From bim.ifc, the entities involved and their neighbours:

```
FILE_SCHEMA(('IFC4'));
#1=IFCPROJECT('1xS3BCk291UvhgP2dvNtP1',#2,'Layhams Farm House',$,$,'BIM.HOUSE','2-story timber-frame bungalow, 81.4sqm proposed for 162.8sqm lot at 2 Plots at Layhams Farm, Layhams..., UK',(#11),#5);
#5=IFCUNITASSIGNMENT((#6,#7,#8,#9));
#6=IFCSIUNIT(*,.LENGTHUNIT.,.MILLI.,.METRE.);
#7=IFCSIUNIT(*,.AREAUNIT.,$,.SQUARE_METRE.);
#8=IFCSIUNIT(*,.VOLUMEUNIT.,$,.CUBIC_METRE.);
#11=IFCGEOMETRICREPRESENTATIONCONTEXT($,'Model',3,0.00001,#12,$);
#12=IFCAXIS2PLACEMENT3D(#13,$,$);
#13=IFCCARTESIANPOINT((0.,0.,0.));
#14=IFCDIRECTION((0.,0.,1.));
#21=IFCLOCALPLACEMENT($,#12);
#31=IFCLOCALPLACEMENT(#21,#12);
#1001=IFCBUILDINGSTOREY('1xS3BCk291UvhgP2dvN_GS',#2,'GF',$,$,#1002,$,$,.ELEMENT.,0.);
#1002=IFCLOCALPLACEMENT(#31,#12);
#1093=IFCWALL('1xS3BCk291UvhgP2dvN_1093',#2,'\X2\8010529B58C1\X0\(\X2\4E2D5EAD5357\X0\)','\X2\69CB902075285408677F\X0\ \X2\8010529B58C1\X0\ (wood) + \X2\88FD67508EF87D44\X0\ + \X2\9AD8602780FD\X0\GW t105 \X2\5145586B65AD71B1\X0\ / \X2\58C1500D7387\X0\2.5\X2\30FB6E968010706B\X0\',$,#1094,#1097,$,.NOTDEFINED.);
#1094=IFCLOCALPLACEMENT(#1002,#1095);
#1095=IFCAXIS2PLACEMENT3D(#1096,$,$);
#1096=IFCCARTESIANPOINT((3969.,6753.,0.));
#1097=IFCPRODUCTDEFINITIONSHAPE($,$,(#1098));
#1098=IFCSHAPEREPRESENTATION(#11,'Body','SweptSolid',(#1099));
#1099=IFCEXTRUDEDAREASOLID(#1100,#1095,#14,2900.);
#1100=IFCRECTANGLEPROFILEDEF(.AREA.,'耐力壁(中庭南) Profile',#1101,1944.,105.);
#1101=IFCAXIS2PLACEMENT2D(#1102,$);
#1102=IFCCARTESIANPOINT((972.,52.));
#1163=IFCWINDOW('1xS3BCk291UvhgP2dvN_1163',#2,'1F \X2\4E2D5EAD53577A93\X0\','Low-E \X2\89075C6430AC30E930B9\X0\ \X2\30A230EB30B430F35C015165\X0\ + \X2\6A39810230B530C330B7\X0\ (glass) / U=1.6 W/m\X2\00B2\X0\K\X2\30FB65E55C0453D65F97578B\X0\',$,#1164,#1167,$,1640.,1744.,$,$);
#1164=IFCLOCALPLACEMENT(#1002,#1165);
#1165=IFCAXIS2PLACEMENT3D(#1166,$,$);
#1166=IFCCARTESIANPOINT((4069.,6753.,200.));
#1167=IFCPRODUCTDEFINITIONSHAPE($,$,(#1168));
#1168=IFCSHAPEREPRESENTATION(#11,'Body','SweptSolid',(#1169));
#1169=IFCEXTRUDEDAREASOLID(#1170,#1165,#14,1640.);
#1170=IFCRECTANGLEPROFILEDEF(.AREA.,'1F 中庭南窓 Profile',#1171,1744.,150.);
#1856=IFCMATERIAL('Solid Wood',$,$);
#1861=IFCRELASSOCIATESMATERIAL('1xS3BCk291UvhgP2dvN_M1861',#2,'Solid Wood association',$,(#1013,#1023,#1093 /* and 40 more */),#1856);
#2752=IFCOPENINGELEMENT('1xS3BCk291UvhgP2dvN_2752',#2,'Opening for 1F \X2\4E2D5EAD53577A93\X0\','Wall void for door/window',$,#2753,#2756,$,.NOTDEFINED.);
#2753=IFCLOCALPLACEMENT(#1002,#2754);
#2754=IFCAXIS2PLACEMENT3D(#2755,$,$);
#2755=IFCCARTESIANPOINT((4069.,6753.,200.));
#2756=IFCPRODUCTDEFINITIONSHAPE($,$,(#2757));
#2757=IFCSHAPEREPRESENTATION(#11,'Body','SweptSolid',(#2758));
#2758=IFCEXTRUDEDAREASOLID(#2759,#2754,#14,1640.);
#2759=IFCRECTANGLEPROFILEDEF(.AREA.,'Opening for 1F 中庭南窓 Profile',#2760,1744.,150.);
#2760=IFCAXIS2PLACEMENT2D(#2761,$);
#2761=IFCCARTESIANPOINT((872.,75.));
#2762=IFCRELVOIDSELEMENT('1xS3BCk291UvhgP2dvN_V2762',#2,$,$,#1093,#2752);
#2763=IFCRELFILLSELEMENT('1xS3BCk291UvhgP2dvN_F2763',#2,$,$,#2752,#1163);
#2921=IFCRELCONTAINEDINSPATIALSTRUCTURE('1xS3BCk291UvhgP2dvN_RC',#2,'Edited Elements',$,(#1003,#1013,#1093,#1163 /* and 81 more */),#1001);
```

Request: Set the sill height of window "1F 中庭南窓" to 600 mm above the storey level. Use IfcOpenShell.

```python
import numpy as np
import ifcopenshell
import ifcopenshell.api.geometry
import ifcopenshell.geom
import ifcopenshell.util.element
import ifcopenshell.util.placement
import ifcopenshell.util.shape
import ifcopenshell.util.unit

model = ifcopenshell.open("bim.ifc")
unit_scale = ifcopenshell.util.unit.calculate_unit_scale(model)

window = model.by_id(1163)
opening = window.FillsVoids[0].RelatingOpeningElement
storey = ifcopenshell.util.element.get_container(window, ifc_class="IfcBuildingStorey")
level = ifcopenshell.util.placement.get_local_placement(storey.ObjectPlacement)[2, 3]

# The opening's origin need not be at the sill, so measure its lowest point.
shape = ifcopenshell.geom.create_shape(ifcopenshell.geom.settings(), opening)
bottom = ifcopenshell.util.shape.get_shape_bottom_elevation(shape, shape.geometry) / unit_scale
dz = level + 600.0 - bottom

shift = np.array([0.0, 0.0, dz])
# The window is not placed relative to its opening, so move both.
for product in (opening, window):
    matrix = ifcopenshell.util.placement.get_local_placement(product.ObjectPlacement)
    matrix[:3, 3] += shift
    ifcopenshell.api.geometry.edit_object_placement(model, product=product, matrix=matrix, is_si=False)

print(f"moved by {dz * unit_scale:+.3f} m")

model.write("bim_rev.ifc")
```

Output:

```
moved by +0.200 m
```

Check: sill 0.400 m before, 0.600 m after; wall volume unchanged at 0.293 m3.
